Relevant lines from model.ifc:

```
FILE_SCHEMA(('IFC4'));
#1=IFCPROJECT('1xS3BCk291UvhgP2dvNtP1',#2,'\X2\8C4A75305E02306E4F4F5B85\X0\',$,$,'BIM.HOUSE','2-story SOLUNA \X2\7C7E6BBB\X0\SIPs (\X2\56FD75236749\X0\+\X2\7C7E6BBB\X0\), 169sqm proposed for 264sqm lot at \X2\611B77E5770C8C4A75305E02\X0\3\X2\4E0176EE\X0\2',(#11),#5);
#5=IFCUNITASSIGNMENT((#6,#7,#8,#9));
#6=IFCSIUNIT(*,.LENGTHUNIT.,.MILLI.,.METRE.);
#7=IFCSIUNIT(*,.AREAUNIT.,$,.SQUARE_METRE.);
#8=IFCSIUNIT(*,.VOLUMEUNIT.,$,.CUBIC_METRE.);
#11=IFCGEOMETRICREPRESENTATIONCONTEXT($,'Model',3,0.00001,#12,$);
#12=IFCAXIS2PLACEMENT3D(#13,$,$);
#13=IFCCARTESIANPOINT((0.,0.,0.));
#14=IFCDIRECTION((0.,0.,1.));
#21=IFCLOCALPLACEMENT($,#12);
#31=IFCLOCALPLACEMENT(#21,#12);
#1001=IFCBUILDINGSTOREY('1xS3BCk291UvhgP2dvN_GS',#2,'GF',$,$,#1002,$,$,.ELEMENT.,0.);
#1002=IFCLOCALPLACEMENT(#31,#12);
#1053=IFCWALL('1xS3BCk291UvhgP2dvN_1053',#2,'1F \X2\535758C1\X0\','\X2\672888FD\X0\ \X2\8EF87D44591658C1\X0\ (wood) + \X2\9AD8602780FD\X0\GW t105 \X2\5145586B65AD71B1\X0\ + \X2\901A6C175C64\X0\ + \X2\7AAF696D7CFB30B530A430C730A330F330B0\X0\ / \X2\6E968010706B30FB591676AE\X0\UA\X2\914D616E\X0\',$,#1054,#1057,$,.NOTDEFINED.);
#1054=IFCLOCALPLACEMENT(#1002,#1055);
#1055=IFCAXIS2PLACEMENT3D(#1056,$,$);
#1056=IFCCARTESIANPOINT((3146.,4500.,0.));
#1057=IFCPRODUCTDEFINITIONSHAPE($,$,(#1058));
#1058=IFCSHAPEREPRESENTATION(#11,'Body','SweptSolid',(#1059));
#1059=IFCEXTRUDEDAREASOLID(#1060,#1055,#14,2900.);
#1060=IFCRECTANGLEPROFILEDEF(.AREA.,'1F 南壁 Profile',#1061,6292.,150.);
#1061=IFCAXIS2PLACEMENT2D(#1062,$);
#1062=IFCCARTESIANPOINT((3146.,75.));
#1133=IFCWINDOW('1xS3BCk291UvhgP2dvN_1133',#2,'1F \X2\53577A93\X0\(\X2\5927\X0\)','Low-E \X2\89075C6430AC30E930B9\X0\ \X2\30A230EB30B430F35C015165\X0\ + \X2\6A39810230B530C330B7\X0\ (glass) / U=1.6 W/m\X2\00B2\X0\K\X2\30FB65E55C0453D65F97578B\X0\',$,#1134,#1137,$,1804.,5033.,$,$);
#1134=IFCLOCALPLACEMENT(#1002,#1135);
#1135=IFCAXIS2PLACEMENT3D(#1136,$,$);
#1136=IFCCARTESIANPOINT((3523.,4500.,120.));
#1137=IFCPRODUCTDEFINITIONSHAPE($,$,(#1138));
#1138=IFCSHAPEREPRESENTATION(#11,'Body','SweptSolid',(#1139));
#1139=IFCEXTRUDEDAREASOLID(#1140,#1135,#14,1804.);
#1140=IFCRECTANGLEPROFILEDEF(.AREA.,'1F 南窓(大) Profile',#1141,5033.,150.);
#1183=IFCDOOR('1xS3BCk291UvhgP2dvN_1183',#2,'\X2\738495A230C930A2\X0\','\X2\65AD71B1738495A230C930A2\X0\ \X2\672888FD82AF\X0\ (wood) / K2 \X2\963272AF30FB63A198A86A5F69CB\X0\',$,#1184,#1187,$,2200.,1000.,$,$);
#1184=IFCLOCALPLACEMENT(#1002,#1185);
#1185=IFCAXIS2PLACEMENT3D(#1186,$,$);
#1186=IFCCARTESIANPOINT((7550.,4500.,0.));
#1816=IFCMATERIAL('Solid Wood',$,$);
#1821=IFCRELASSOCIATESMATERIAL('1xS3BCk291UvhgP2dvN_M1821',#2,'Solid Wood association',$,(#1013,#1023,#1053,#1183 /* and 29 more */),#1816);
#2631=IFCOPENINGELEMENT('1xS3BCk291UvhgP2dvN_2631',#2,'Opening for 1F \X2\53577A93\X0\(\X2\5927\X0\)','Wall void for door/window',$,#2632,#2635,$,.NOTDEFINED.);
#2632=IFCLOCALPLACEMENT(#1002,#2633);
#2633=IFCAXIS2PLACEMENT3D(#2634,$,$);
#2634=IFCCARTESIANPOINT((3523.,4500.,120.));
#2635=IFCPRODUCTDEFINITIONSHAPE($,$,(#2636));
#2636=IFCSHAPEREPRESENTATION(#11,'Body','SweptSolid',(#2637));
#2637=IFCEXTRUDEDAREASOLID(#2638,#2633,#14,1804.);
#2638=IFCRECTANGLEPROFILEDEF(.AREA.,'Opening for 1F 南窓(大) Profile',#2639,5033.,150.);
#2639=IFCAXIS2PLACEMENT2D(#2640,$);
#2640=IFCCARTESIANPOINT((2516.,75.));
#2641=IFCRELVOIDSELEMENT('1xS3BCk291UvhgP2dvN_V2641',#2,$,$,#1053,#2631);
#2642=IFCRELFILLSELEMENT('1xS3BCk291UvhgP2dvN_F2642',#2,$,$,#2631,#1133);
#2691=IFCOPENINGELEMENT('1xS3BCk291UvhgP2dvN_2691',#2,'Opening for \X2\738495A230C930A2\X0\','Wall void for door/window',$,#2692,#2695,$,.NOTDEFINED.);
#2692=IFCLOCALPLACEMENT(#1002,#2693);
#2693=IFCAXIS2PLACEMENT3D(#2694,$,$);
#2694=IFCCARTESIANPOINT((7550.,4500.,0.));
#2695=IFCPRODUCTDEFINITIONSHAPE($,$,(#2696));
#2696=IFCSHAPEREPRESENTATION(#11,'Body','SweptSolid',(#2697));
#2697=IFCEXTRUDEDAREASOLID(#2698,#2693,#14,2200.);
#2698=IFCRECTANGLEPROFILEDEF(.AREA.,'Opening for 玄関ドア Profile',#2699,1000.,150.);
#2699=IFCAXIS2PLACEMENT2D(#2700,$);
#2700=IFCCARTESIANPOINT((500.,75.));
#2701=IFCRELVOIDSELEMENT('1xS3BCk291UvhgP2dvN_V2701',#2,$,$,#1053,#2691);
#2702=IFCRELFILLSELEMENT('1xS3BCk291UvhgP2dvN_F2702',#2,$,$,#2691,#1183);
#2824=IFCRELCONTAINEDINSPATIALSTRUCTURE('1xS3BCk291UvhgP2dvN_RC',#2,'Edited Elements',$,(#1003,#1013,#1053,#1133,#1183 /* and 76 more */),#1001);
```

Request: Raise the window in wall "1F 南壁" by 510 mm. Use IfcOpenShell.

```python
import numpy as np
import ifcopenshell
import ifcopenshell.api.geometry
import ifcopenshell.util.placement
import ifcopenshell.util.unit

model = ifcopenshell.open("model.ifc")
unit_scale = ifcopenshell.util.unit.calculate_unit_scale(model)

window = model.by_id(1133)
opening = window.FillsVoids[0].RelatingOpeningElement
dz = 0.51 / unit_scale

shift = np.array([0.0, 0.0, dz])
# The window is not placed relative to its opening, so move both.
for product in (opening, window):
    matrix = ifcopenshell.util.placement.get_local_placement(product.ObjectPlacement)
    matrix[:3, 3] += shift
    ifcopenshell.api.geometry.edit_object_placement(model, product=product, matrix=matrix, is_si=False)

print(f"moved by {dz * unit_scale:+.3f} m")

model.write("model_edited.ifc")
```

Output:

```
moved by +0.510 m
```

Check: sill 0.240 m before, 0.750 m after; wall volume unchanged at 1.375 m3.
